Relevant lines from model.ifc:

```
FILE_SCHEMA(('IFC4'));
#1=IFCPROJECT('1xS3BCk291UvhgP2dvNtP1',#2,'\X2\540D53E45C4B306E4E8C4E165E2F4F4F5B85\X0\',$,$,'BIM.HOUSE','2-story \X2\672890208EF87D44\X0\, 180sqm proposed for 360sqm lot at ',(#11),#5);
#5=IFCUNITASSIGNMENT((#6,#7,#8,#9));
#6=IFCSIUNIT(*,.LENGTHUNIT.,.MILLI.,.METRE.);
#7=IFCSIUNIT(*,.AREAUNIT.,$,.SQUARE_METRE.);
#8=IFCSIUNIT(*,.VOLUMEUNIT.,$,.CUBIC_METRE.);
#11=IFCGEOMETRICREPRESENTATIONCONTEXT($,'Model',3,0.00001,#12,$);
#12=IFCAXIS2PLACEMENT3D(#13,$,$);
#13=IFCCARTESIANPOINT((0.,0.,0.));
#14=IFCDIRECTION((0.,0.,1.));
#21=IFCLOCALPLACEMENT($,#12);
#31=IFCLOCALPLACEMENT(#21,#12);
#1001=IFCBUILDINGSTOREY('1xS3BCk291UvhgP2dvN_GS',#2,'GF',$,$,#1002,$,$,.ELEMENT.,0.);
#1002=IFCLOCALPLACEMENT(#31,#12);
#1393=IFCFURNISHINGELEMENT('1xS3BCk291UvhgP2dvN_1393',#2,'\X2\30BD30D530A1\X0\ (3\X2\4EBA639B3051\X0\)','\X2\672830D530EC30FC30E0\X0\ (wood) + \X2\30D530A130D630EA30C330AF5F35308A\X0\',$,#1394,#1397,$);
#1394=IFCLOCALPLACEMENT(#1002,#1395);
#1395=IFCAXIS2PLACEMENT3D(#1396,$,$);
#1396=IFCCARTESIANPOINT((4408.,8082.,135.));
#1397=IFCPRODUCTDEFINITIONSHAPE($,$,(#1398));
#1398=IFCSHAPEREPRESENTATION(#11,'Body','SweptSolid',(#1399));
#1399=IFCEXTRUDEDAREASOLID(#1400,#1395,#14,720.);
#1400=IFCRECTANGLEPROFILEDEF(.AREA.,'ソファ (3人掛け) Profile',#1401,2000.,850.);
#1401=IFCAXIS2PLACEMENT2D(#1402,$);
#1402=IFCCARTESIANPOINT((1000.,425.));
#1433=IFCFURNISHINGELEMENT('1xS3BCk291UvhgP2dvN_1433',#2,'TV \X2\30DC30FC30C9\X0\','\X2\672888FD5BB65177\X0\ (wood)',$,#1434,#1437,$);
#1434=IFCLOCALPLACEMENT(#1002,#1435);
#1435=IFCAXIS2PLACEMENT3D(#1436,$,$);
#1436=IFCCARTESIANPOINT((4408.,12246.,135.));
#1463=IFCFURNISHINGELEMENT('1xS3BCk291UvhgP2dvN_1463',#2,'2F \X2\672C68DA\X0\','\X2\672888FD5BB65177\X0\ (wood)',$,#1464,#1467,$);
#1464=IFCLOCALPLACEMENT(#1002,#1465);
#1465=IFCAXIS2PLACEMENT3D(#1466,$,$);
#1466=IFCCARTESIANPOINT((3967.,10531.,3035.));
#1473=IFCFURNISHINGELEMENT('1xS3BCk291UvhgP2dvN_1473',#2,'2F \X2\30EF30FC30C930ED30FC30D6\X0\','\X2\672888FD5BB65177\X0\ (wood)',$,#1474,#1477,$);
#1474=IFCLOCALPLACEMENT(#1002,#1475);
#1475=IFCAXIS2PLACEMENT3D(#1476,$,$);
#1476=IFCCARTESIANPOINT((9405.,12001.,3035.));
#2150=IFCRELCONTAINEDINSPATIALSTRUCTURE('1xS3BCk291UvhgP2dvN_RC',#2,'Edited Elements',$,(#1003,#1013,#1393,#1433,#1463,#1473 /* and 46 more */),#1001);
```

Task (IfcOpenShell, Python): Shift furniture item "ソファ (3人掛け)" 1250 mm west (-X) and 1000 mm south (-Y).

```python
import ifcopenshell
import ifcopenshell.api.geometry
import ifcopenshell.util.placement
import ifcopenshell.util.unit

model = ifcopenshell.open("model.ifc")
unit_scale = ifcopenshell.util.unit.calculate_unit_scale(model)

item = model.by_guid("1xS3BCk291UvhgP2dvN_1393")
matrix = ifcopenshell.util.placement.get_local_placement(item.ObjectPlacement)
matrix[0, 3] -= 1.25 / unit_scale
matrix[1, 3] -= 1 / unit_scale
ifcopenshell.api.geometry.edit_object_placement(model, product=item, matrix=matrix, is_si=False)

print(ifcopenshell.util.placement.get_local_placement(item.ObjectPlacement).round(3) + 0.0)

model.write("model_v2.ifc")
```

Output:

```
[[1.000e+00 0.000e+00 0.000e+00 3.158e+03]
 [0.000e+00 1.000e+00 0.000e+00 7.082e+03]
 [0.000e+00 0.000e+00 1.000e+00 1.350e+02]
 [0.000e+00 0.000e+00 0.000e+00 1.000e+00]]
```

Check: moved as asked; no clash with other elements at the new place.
